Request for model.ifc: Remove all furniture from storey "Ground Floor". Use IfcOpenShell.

First a look at what the model holds.

```python
import ifcopenshell
import ifcopenshell.util.element

model = ifcopenshell.open("model.ifc")
print(model.schema)
storey = next(s for s in model.by_type("IfcBuildingStorey") if s.Name == "Ground Floor")
furniture = [e for e in ifcopenshell.util.element.get_decomposition(storey) if e.is_a("IfcFurnishingElement")]
seen = {}
for e in furniture:
    element_type = ifcopenshell.util.element.get_type(e)
    name = element_type.Name if element_type not in (None, e) else None
    seen[name] = seen.get(name, 0) + 1
for name, count in sorted(seen.items(), key=str):
    print(count, "x", name)
```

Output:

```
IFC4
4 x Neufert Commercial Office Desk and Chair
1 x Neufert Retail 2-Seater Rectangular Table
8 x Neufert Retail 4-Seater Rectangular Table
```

```python
import ifcopenshell
import ifcopenshell.api.root
import ifcopenshell.util.element

model = ifcopenshell.open("model.ifc")

storey = next(s for s in model.by_type("IfcBuildingStorey") if s.Name == "Ground Floor")
furniture = [e for e in ifcopenshell.util.element.get_decomposition(storey) if e.is_a("IfcFurnishingElement")]

for e in furniture:
    ifcopenshell.api.root.remove_product(model, product=e)
print(len(furniture), "removed")

model.write("model_v2.ifc")
```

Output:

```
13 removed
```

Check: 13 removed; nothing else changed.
